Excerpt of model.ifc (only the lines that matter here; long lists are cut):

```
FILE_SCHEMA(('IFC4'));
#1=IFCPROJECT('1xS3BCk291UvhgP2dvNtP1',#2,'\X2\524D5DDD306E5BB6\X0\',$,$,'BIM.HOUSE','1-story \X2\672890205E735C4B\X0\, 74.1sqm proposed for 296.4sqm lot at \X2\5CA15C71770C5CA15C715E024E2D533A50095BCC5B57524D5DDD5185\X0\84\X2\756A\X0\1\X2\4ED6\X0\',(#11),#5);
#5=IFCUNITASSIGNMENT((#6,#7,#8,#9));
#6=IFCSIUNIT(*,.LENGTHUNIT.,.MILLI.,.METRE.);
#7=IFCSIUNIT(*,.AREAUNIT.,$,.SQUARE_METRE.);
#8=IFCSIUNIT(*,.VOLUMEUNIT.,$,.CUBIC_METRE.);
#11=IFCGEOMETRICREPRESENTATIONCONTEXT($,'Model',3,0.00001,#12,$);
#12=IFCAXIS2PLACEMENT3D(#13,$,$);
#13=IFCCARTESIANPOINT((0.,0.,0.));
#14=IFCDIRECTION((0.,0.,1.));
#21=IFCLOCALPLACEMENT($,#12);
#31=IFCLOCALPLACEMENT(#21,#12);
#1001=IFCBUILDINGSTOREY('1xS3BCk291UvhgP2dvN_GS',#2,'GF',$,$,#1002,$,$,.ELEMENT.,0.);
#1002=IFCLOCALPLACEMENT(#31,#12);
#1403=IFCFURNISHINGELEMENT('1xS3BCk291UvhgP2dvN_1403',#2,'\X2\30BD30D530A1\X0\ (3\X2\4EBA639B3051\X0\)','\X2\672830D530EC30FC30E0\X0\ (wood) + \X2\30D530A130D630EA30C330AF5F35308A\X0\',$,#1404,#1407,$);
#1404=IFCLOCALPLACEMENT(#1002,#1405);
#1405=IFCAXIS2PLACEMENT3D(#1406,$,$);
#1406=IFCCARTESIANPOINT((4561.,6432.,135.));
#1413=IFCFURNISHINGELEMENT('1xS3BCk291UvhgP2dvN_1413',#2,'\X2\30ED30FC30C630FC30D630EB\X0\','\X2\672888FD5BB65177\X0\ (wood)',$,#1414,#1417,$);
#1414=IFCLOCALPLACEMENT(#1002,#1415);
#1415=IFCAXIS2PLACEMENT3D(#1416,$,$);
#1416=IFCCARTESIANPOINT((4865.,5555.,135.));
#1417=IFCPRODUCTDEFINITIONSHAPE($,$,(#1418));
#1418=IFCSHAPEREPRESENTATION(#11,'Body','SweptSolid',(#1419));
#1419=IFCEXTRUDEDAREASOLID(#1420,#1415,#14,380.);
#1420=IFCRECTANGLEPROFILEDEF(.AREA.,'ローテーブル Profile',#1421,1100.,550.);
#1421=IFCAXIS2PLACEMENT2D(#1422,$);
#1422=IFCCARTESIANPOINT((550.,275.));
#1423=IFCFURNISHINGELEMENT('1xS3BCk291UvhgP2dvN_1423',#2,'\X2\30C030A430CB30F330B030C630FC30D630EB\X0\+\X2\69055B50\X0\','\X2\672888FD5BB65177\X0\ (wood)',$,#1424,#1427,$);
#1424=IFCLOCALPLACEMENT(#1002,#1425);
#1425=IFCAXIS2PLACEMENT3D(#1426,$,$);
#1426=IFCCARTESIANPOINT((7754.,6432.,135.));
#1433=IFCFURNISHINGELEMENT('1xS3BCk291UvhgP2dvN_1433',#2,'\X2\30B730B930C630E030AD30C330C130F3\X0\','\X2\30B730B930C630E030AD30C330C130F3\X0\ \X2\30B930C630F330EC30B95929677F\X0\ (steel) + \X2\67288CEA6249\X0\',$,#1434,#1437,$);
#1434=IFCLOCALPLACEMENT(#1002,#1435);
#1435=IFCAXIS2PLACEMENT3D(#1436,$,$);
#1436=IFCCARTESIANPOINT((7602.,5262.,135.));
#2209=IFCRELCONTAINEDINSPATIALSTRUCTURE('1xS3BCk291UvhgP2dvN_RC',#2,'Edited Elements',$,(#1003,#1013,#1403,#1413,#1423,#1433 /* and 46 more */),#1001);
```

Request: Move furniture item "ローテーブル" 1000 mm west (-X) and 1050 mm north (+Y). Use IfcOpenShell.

```python
import ifcopenshell
import ifcopenshell.api.geometry
import ifcopenshell.util.placement
import ifcopenshell.util.unit

model = ifcopenshell.open("model.ifc")
unit_scale = ifcopenshell.util.unit.calculate_unit_scale(model)

item = model.by_guid("1xS3BCk291UvhgP2dvN_1413")
matrix = ifcopenshell.util.placement.get_local_placement(item.ObjectPlacement)
matrix[0, 3] -= 1 / unit_scale
matrix[1, 3] += 1.05 / unit_scale
ifcopenshell.api.geometry.edit_object_placement(model, product=item, matrix=matrix, is_si=False)

print(ifcopenshell.util.placement.get_local_placement(item.ObjectPlacement).round(3) + 0.0)

model.write("model-out.ifc")
```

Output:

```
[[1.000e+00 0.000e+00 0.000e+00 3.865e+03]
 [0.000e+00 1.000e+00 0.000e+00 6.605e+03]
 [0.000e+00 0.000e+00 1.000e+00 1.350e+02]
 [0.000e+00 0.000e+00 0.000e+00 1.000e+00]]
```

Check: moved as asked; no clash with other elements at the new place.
